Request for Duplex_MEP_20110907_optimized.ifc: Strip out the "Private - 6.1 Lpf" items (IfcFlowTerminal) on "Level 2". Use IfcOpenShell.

First a look at what the model holds.

```python
import ifcopenshell
import ifcopenshell.util.element

model = ifcopenshell.open("Duplex_MEP_20110907_optimized.ifc")
print(model.schema)
storey = next(s for s in model.by_type("IfcBuildingStorey") if s.Name == "Level 2")
terminals = [e for e in ifcopenshell.util.element.get_decomposition(storey) if e.is_a("IfcFlowTerminal")]
seen = {}
for e in terminals:
    element_type = ifcopenshell.util.element.get_type(e)
    name = element_type.Name if element_type not in (None, e) else None
    seen[name] = seen.get(name, 0) + 1
for name, count in sorted(seen.items(), key=str):
    print(count, "x", name)
```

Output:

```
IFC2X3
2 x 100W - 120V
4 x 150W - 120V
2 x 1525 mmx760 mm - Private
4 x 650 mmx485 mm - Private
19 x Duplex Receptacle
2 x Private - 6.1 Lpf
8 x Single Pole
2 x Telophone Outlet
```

```python
import ifcopenshell
import ifcopenshell.api.root
import ifcopenshell.util.element

model = ifcopenshell.open("Duplex_MEP_20110907_optimized.ifc")

storey = next(s for s in model.by_type("IfcBuildingStorey") if s.Name == "Level 2")
terminals = [e for e in ifcopenshell.util.element.get_decomposition(storey) if e.is_a("IfcFlowTerminal")]
targets = [e for e in terminals if (t := ifcopenshell.util.element.get_type(e)) not in (None, e) and t.Name == "Private - 6.1 Lpf"]

for e in targets:
    ifcopenshell.api.root.remove_product(model, product=e)
print(len(targets), "removed")

model.write("Duplex_MEP_20110907_optimized_updated.ifc")
```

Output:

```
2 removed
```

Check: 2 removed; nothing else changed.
